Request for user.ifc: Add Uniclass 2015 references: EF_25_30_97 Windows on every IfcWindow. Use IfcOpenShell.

First a look at what the model holds.

```python
import ifcopenshell

model = ifcopenshell.open("user.ifc")
print(model.schema)
print("classifications:", [c.Name for c in model.by_type("IfcClassification")])
for ifc_class in ("IfcDoor", "IfcRoof", "IfcStair", "IfcWall", "IfcWindow"):
    print(ifc_class, len(model.by_type(ifc_class)))
```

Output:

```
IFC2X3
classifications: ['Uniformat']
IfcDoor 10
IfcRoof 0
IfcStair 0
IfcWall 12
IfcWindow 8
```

```python
import ifcopenshell
import ifcopenshell.api.classification

model = ifcopenshell.open("user.ifc")

# IFC2X3 requires Source and Edition and has no link from the project to the system.
system = model.create_entity("IfcClassification", Source="NBS", Edition="2015", Name="Uniclass 2015")

codes = {
    "IfcWindow": ("EF_25_30_97", "Windows"),
}
for ifc_class, (code, name) in codes.items():
    products = model.by_type(ifc_class)
    ifcopenshell.api.classification.add_reference(
        model, products=products, classification=system, identification=code, name=name
    )
    print(code, len(products))

model.write("user_rev.ifc")
```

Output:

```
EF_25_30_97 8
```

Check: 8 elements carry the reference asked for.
